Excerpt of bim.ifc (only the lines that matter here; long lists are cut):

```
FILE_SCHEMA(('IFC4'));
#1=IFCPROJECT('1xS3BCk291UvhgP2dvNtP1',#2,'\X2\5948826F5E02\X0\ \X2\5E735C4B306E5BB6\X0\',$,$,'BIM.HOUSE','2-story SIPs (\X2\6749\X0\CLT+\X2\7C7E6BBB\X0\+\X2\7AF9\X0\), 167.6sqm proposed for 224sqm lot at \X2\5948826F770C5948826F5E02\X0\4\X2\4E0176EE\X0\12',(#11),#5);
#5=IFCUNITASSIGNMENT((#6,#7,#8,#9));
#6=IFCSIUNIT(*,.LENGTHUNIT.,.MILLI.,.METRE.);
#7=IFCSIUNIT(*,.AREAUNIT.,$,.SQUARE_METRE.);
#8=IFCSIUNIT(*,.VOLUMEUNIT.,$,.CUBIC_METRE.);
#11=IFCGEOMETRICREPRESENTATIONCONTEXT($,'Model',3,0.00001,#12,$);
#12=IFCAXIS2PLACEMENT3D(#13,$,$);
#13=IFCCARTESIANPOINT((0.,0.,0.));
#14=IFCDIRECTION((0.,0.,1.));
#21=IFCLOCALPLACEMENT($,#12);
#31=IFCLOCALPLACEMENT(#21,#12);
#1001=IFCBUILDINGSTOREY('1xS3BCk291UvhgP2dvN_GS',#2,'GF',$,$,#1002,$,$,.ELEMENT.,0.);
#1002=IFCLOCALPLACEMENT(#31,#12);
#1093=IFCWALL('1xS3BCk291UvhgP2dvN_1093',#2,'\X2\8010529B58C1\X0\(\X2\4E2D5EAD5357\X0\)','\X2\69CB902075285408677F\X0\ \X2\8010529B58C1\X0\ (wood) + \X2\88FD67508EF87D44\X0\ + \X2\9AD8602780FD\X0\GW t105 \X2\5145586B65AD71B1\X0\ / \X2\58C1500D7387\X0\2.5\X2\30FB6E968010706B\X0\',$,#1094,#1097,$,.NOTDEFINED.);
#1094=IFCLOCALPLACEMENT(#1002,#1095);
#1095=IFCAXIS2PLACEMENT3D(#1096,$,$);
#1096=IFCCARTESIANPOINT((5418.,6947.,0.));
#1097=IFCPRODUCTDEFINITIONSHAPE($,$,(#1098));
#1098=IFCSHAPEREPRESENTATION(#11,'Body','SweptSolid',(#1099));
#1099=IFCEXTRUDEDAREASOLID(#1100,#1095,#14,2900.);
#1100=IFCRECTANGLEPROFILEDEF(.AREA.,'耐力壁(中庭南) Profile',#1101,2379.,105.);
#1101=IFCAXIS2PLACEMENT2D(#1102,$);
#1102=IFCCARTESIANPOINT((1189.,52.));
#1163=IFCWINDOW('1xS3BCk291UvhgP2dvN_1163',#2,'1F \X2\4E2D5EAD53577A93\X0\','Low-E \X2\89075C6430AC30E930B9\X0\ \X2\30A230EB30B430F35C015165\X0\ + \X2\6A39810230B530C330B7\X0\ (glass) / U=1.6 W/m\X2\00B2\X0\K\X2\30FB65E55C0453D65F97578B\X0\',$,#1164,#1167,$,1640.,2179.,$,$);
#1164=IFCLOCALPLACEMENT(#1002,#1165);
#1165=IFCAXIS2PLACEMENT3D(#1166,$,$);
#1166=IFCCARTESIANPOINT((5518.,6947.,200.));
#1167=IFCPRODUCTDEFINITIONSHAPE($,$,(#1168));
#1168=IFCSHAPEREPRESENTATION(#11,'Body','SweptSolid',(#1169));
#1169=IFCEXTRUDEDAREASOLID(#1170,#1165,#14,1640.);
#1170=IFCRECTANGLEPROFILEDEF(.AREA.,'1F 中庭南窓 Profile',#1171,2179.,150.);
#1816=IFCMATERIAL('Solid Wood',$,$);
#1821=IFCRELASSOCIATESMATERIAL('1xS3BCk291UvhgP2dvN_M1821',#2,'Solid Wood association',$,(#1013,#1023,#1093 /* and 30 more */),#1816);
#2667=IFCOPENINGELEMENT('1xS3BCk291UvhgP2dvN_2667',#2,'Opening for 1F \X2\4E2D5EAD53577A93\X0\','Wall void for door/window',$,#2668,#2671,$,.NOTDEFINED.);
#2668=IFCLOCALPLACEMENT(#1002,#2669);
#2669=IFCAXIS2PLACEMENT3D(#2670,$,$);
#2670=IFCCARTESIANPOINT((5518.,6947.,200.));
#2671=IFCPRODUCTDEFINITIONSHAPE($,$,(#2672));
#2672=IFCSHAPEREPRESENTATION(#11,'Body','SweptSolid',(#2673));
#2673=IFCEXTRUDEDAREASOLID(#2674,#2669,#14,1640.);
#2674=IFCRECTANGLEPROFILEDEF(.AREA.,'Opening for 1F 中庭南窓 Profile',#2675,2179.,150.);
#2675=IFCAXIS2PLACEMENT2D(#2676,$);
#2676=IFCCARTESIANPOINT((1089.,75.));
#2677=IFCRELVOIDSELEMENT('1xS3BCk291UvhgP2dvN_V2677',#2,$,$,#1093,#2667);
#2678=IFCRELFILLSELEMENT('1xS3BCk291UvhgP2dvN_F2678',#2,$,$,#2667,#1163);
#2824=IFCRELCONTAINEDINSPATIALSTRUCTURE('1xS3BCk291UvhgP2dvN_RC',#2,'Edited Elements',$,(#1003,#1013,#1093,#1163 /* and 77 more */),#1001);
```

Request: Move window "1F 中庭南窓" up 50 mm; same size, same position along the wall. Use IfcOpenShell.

```python
import numpy as np
import ifcopenshell
import ifcopenshell.api.geometry
import ifcopenshell.util.placement
import ifcopenshell.util.unit

model = ifcopenshell.open("bim.ifc")
unit_scale = ifcopenshell.util.unit.calculate_unit_scale(model)

window = model.by_id(1163)
opening = window.FillsVoids[0].RelatingOpeningElement
dz = 50.0

shift = np.array([0.0, 0.0, dz])
# The window is not placed relative to its opening, so move both.
for product in (opening, window):
    matrix = ifcopenshell.util.placement.get_local_placement(product.ObjectPlacement)
    matrix[:3, 3] += shift
    ifcopenshell.api.geometry.edit_object_placement(model, product=product, matrix=matrix, is_si=False)

print(f"moved by {dz * unit_scale:+.3f} m")

model.write("bim_v2.ifc")
```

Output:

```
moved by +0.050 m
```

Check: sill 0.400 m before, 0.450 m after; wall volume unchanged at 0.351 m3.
